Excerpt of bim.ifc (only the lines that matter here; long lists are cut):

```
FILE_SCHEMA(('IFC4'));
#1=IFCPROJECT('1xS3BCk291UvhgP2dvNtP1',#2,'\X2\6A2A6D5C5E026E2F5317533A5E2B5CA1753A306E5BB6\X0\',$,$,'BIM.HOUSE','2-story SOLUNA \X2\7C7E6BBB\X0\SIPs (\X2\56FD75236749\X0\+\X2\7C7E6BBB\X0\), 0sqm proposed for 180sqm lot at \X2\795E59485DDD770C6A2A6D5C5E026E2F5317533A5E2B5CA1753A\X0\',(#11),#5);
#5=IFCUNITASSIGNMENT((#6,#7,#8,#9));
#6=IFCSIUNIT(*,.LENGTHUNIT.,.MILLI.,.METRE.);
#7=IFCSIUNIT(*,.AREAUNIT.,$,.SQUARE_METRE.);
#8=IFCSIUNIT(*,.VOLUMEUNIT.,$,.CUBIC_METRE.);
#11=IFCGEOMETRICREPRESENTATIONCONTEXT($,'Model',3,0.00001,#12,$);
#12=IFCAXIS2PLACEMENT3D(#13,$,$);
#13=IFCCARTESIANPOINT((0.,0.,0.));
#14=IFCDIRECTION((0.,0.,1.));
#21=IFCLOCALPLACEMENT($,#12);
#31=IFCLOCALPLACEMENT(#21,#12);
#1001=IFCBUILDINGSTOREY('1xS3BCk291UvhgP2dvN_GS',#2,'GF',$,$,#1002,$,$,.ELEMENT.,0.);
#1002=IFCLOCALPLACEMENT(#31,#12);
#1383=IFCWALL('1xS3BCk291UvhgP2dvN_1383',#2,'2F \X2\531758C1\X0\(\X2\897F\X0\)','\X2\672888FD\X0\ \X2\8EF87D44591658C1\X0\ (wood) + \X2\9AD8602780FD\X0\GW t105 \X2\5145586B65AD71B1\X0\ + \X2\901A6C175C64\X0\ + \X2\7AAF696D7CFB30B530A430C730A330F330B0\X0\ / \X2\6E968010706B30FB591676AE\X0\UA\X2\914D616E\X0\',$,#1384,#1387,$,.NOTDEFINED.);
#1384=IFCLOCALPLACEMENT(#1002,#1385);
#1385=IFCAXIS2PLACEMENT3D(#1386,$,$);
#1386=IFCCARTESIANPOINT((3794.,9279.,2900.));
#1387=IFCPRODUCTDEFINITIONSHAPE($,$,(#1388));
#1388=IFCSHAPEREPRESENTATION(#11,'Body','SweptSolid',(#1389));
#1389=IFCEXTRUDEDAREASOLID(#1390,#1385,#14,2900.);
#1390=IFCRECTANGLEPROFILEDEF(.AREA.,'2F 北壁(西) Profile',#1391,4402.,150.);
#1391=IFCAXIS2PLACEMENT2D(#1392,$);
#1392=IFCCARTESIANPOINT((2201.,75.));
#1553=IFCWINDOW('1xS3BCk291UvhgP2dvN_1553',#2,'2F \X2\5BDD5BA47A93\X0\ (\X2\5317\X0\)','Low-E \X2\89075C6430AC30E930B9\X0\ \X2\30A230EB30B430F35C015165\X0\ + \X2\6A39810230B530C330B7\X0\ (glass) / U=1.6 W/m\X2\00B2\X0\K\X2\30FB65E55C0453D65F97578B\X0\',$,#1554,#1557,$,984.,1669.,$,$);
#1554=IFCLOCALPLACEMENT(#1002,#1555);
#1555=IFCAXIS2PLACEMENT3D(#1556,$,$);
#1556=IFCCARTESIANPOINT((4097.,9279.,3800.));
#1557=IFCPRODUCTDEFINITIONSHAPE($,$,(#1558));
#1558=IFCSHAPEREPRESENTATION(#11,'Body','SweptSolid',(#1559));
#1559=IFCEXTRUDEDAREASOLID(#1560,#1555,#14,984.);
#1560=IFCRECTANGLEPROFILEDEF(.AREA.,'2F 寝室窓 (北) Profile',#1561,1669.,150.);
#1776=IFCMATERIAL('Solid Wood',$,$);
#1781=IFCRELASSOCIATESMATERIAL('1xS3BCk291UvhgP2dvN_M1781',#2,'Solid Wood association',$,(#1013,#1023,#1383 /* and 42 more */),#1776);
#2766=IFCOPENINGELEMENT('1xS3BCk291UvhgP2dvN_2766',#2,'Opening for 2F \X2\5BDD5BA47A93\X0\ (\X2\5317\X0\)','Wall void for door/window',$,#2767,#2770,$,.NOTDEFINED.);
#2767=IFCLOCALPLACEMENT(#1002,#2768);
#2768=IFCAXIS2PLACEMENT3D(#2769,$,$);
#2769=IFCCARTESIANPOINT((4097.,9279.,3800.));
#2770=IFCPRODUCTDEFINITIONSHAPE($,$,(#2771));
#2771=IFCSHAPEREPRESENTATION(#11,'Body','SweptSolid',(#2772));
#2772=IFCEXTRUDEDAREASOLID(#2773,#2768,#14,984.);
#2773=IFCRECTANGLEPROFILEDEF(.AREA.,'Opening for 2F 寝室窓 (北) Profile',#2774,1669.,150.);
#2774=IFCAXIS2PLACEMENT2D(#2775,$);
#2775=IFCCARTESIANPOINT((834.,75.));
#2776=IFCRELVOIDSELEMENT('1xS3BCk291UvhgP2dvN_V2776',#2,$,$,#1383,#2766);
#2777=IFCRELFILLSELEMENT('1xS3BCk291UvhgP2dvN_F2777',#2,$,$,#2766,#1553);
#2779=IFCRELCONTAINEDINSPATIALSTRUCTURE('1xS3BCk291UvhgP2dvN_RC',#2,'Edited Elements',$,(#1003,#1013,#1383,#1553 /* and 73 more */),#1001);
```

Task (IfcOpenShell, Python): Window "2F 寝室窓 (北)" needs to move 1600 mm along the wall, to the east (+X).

```python
import ifcopenshell
import ifcopenshell.api.geometry
import ifcopenshell.util.placement
import ifcopenshell.util.unit

model = ifcopenshell.open("bim.ifc")
unit_scale = ifcopenshell.util.unit.calculate_unit_scale(model)

window = model.by_guid("1xS3BCk291UvhgP2dvN_1553")
opening = window.FillsVoids[0].RelatingOpeningElement
wall = opening.VoidsElements[0].RelatingBuildingElement

wall_matrix = ifcopenshell.util.placement.get_local_placement(wall.ObjectPlacement)
shift = wall_matrix[:3, 0] * 1.6 / unit_scale
before = ifcopenshell.util.placement.get_local_placement(window.ObjectPlacement)[:3, 3].copy()

# The window is not placed relative to its opening, so move both.
for product in (opening, window):
    matrix = ifcopenshell.util.placement.get_local_placement(product.ObjectPlacement)
    matrix[:3, 3] += shift
    ifcopenshell.api.geometry.edit_object_placement(model, product=product, matrix=matrix, is_si=False)

after = ifcopenshell.util.placement.get_local_placement(window.ObjectPlacement)[:3, 3]
print("window moved by", (after - before).round(3) + 0.0)

model.write("bim_updated.ifc")
```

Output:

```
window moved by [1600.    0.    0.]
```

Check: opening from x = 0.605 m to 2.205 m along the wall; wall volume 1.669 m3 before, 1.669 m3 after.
